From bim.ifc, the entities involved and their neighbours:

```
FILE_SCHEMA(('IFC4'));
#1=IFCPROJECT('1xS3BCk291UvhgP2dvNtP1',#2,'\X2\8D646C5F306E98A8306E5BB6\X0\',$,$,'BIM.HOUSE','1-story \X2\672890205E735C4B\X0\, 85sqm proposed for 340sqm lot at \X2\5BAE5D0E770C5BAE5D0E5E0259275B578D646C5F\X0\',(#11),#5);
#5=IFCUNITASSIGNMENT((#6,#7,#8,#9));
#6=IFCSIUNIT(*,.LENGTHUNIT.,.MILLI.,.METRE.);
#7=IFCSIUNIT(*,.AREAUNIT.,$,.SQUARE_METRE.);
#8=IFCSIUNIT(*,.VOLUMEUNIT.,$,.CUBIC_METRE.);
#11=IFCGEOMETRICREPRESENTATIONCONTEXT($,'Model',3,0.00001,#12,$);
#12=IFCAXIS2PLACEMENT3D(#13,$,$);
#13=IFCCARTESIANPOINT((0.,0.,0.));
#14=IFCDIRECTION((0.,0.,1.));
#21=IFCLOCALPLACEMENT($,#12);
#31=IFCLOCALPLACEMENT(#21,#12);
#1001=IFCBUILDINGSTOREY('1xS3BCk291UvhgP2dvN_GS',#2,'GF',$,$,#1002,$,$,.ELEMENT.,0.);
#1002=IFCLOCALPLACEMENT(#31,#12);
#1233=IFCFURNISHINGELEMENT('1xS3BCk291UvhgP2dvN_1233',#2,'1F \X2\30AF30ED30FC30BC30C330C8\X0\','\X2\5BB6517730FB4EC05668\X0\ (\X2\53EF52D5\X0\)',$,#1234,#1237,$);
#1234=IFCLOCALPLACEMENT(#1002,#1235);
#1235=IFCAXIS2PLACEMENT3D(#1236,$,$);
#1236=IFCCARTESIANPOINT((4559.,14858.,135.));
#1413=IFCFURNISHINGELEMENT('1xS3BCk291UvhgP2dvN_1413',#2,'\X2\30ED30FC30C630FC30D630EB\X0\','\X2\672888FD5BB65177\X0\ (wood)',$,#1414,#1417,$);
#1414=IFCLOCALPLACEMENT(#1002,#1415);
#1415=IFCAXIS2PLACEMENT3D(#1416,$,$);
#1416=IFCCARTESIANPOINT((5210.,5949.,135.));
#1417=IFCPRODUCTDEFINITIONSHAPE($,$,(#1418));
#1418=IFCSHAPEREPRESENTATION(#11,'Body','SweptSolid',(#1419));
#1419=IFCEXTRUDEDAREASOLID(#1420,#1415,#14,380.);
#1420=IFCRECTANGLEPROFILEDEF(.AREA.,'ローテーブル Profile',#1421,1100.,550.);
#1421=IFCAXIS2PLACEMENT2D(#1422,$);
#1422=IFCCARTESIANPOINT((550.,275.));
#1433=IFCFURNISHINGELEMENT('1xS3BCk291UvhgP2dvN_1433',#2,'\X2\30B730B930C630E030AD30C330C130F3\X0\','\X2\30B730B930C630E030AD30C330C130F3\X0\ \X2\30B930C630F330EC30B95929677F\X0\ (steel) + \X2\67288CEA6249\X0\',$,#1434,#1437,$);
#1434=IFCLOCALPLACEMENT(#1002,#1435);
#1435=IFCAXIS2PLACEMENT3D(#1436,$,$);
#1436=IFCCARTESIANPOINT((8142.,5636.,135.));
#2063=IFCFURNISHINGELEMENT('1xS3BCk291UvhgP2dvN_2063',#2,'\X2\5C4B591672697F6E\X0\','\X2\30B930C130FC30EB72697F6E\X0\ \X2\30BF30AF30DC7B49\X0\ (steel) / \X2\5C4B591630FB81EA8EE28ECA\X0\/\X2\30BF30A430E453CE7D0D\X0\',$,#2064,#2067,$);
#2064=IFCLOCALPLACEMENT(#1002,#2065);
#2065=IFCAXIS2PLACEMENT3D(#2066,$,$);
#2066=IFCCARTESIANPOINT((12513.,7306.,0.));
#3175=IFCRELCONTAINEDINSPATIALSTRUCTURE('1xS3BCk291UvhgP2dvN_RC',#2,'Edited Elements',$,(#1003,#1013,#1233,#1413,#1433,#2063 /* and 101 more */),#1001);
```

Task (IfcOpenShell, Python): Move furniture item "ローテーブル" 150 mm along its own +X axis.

```python
import ifcopenshell
import ifcopenshell.api.geometry
import ifcopenshell.util.placement
import ifcopenshell.util.unit

model = ifcopenshell.open("bim.ifc")
unit_scale = ifcopenshell.util.unit.calculate_unit_scale(model)

item = model.by_guid("1xS3BCk291UvhgP2dvN_1413")
matrix = ifcopenshell.util.placement.get_local_placement(item.ObjectPlacement)
matrix[:3, 3] += matrix[:3, 0] * 0.15 / unit_scale
ifcopenshell.api.geometry.edit_object_placement(model, product=item, matrix=matrix, is_si=False)

print(ifcopenshell.util.placement.get_local_placement(item.ObjectPlacement).round(3) + 0.0)

model.write("bim_edited.ifc")
```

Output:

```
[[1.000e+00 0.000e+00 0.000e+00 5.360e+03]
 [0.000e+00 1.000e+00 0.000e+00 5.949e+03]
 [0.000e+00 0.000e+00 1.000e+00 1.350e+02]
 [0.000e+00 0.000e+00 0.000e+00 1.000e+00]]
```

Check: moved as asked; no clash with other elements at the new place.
